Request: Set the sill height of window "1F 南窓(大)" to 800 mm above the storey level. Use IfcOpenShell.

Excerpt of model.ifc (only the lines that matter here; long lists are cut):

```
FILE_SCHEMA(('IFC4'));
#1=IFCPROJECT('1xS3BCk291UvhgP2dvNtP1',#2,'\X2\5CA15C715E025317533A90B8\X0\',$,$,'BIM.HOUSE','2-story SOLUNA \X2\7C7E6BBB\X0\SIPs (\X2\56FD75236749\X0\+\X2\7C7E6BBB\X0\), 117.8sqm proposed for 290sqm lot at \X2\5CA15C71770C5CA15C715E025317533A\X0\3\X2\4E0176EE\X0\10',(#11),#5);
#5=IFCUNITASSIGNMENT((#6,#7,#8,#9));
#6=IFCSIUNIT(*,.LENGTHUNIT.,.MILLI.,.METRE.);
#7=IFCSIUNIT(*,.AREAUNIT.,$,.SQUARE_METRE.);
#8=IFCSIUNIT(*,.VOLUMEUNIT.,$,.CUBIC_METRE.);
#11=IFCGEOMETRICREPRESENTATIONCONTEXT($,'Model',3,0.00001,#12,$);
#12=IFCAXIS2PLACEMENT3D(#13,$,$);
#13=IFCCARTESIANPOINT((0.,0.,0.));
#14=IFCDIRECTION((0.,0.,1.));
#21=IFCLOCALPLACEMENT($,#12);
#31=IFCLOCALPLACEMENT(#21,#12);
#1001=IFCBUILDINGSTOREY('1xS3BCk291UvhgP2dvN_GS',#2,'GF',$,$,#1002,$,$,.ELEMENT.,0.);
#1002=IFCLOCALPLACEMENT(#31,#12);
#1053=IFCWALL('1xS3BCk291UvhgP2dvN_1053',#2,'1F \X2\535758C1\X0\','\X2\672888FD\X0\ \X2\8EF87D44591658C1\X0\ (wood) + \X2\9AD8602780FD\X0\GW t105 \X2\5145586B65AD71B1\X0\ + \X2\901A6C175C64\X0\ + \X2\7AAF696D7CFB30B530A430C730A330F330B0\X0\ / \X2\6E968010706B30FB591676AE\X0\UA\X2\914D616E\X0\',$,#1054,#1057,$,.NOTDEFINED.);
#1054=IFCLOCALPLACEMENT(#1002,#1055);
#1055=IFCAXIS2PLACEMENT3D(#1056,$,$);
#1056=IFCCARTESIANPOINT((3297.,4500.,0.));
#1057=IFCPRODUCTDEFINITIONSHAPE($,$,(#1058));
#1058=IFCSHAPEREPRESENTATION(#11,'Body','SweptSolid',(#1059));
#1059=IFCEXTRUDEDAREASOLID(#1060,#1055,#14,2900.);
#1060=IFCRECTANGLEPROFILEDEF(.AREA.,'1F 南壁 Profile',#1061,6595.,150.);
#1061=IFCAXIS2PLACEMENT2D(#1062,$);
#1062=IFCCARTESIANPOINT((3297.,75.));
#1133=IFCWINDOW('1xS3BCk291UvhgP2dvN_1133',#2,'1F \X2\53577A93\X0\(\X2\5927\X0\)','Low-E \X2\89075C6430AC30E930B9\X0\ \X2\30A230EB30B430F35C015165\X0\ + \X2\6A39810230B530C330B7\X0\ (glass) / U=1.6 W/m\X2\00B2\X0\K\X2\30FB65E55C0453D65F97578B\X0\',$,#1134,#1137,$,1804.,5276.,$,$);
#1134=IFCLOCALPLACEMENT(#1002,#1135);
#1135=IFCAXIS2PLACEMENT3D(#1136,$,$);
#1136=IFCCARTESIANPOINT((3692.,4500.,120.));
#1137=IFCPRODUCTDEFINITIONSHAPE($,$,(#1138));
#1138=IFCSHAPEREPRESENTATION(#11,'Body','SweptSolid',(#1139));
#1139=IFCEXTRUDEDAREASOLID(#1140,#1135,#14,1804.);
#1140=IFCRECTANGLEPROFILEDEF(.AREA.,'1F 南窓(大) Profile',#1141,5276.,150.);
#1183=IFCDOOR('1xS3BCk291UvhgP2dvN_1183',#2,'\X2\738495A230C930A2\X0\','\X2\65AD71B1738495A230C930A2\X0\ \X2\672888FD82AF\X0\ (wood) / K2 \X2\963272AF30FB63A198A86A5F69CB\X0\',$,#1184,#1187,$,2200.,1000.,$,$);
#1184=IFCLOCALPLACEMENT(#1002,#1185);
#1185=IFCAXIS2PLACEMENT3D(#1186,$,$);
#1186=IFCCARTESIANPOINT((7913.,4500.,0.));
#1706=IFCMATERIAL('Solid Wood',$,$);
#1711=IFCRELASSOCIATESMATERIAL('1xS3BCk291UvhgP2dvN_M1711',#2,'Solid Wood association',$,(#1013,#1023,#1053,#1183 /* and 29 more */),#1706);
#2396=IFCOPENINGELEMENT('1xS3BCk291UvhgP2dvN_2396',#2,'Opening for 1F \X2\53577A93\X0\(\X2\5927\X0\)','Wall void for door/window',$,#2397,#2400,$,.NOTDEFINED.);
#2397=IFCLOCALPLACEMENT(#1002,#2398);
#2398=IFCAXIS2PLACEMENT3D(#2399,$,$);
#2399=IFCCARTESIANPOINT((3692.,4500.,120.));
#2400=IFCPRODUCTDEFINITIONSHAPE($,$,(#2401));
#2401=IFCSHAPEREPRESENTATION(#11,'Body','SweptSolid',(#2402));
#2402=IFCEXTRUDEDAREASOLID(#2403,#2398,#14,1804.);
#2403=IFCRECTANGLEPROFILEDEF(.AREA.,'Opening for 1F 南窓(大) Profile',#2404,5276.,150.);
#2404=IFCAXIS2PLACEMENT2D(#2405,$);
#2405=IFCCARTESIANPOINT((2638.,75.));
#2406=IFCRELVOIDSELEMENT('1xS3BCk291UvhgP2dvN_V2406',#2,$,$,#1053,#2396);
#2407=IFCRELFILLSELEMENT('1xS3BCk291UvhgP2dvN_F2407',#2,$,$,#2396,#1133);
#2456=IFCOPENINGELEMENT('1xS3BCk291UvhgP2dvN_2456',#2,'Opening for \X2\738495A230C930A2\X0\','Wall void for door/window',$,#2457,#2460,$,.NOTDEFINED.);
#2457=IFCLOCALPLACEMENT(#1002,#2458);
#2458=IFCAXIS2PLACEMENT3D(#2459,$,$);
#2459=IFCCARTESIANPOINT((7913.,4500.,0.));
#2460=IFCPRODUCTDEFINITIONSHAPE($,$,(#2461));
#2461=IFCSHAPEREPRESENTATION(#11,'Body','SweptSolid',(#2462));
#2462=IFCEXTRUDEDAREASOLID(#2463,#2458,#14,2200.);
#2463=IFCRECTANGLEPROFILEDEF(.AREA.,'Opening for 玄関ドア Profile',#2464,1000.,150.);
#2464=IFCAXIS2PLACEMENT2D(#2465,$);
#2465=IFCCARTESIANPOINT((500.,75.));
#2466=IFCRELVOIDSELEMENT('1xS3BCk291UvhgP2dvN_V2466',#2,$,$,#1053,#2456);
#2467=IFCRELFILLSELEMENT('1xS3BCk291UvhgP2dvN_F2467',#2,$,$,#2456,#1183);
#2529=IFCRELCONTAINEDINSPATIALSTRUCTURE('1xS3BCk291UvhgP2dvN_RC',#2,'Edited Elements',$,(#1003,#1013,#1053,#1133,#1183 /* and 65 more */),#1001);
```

```python
import numpy as np
import ifcopenshell
import ifcopenshell.api.geometry
import ifcopenshell.geom
import ifcopenshell.util.element
import ifcopenshell.util.placement
import ifcopenshell.util.shape
import ifcopenshell.util.unit

model = ifcopenshell.open("model.ifc")
unit_scale = ifcopenshell.util.unit.calculate_unit_scale(model)

window = model.by_guid("1xS3BCk291UvhgP2dvN_1133")
opening = window.FillsVoids[0].RelatingOpeningElement
storey = ifcopenshell.util.element.get_container(window, ifc_class="IfcBuildingStorey")
level = ifcopenshell.util.placement.get_local_placement(storey.ObjectPlacement)[2, 3]

# The opening's origin need not be at the sill, so measure its lowest point.
shape = ifcopenshell.geom.create_shape(ifcopenshell.geom.settings(), opening)
bottom = ifcopenshell.util.shape.get_shape_bottom_elevation(shape, shape.geometry) / unit_scale
dz = level + 800.0 - bottom

shift = np.array([0.0, 0.0, dz])
# The window is not placed relative to its opening, so move both.
for product in (opening, window):
    matrix = ifcopenshell.util.placement.get_local_placement(product.ObjectPlacement)
    matrix[:3, 3] += shift
    ifcopenshell.api.geometry.edit_object_placement(model, product=product, matrix=matrix, is_si=False)

print(f"moved by {dz * unit_scale:+.3f} m")

model.write("model_rev.ifc")
```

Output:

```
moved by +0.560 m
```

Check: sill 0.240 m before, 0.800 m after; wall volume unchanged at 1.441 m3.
